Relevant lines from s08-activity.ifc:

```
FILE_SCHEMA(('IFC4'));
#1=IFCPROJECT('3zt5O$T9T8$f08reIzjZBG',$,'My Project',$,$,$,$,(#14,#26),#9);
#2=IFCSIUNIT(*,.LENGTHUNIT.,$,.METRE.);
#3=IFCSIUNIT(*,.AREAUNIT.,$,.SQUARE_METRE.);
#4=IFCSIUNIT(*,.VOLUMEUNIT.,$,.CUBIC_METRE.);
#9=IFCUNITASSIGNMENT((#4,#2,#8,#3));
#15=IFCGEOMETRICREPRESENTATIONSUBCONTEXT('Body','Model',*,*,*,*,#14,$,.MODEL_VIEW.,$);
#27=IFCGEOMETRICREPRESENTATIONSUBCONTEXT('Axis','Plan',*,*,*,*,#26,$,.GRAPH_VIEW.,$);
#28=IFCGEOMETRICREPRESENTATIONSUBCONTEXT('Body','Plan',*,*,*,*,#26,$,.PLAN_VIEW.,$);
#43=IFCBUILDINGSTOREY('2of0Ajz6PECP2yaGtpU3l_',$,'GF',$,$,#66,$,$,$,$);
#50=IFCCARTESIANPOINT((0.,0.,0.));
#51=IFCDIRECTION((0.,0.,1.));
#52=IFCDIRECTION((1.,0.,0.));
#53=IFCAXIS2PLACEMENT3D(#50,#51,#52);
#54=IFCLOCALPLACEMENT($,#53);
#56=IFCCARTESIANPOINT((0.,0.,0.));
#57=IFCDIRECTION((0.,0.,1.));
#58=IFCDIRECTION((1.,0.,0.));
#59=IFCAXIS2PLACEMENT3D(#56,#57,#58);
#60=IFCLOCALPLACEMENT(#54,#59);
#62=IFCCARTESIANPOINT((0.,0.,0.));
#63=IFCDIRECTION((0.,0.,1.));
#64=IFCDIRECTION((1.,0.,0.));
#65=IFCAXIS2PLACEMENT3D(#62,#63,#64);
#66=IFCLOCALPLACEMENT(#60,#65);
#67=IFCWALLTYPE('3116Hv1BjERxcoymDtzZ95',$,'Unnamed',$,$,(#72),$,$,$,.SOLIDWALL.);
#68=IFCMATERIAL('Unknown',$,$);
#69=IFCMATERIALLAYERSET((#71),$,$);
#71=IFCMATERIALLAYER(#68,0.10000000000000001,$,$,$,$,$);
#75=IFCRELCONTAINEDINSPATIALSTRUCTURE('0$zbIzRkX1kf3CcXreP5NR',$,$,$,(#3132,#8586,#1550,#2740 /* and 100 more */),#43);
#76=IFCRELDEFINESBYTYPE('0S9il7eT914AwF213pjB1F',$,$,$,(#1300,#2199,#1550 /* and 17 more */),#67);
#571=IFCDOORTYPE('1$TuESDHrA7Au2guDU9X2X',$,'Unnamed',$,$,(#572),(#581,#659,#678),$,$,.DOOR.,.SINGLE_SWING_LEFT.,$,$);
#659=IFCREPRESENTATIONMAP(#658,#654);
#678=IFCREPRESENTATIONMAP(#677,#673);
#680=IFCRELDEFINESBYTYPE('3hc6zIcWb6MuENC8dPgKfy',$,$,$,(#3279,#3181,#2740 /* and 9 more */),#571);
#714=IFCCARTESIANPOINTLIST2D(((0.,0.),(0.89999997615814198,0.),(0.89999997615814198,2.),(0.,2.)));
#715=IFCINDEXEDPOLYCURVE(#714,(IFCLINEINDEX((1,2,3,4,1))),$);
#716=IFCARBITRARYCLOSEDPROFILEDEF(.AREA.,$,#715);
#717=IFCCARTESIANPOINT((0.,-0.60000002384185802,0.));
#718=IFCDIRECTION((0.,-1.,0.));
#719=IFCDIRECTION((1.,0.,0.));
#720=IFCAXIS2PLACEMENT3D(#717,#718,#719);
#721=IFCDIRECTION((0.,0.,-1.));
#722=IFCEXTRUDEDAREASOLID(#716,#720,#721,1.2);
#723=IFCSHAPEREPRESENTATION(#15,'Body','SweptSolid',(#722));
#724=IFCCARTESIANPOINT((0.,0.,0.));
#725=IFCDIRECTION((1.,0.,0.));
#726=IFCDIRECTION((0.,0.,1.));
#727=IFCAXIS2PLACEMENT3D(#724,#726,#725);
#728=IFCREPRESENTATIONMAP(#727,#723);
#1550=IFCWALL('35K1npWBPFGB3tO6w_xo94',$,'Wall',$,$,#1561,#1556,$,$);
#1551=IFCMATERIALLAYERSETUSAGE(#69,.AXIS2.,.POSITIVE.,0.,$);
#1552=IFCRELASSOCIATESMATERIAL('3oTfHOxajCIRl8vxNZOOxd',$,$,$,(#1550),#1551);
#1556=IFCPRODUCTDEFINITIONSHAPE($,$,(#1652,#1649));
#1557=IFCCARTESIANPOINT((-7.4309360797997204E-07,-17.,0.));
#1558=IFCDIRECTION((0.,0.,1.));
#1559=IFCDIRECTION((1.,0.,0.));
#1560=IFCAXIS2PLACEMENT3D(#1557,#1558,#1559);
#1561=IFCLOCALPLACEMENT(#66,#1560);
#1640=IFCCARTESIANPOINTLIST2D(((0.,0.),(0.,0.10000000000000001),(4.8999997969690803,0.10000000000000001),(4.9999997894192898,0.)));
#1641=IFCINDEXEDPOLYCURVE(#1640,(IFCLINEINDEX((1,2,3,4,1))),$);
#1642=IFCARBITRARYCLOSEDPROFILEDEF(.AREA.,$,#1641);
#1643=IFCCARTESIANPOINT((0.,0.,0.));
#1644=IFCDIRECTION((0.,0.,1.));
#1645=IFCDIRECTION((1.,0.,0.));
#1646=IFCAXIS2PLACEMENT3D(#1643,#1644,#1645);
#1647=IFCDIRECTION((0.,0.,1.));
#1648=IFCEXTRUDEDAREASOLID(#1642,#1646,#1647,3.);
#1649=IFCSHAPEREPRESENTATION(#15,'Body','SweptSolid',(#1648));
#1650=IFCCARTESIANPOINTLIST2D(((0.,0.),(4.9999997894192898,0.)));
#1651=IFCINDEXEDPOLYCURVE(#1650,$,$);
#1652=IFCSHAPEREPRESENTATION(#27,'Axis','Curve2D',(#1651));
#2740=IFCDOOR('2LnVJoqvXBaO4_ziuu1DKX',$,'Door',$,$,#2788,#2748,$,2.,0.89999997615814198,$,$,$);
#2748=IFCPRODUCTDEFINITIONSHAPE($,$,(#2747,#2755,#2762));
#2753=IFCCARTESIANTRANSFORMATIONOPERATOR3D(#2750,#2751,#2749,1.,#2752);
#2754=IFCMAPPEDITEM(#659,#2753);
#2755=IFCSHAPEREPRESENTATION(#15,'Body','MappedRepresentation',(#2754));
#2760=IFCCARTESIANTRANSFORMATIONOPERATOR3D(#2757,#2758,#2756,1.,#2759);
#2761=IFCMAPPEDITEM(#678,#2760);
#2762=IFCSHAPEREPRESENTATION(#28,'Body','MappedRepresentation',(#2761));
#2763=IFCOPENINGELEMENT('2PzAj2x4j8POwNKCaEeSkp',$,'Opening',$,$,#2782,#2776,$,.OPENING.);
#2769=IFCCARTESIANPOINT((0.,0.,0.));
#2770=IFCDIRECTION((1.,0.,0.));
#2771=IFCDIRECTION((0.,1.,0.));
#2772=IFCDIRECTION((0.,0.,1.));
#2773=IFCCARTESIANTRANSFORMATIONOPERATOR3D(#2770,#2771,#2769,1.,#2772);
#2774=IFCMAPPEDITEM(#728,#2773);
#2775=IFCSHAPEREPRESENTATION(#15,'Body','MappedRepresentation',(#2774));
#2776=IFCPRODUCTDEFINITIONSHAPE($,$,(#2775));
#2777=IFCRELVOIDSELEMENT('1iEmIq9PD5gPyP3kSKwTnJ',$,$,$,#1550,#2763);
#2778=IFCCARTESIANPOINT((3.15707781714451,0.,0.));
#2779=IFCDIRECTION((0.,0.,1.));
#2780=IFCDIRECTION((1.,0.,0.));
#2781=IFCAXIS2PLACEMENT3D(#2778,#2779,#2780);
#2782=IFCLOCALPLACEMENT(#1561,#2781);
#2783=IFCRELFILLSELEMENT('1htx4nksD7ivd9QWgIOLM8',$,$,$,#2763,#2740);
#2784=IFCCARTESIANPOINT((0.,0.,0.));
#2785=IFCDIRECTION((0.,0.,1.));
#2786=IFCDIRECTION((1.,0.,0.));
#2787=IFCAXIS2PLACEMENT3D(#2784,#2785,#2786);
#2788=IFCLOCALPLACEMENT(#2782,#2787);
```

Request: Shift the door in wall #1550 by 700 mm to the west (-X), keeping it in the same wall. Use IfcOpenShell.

```python
import ifcopenshell
import ifcopenshell.api.geometry
import ifcopenshell.util.placement

model = ifcopenshell.open("s08-activity.ifc")

door = model.by_guid("2LnVJoqvXBaO4_ziuu1DKX")
opening = door.FillsVoids[0].RelatingOpeningElement
wall = opening.VoidsElements[0].RelatingBuildingElement

wall_matrix = ifcopenshell.util.placement.get_local_placement(wall.ObjectPlacement)
shift = wall_matrix[:3, 0] * -0.7
before = ifcopenshell.util.placement.get_local_placement(door.ObjectPlacement)[:3, 3].copy()

# The door is placed relative to its opening, so it follows when the opening moves.
matrix = ifcopenshell.util.placement.get_local_placement(opening.ObjectPlacement)
matrix[:3, 3] += shift
ifcopenshell.api.geometry.edit_object_placement(
    model, product=opening, matrix=matrix, is_si=False, should_transform_children=True
)

after = ifcopenshell.util.placement.get_local_placement(door.ObjectPlacement)[:3, 3]
print("door moved by", (after - before).round(3) + 0.0)

model.write("s08-activity_updated.ifc")
```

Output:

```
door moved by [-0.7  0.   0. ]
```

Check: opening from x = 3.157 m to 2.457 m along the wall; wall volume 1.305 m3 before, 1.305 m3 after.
